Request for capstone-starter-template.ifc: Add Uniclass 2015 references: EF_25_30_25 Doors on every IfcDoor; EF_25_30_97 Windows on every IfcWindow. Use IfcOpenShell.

First a look at what the model holds.

```python
import ifcopenshell

model = ifcopenshell.open("capstone-starter-template.ifc")
print(model.schema)
print("classifications:", [c.Name for c in model.by_type("IfcClassification")])
for ifc_class in ("IfcDoor", "IfcRoof", "IfcStair", "IfcWall", "IfcWindow"):
    print(ifc_class, len(model.by_type(ifc_class)))
```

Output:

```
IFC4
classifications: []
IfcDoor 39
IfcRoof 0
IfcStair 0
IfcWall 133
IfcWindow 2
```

```python
import ifcopenshell
import ifcopenshell.api.classification

model = ifcopenshell.open("capstone-starter-template.ifc")

system = ifcopenshell.api.classification.add_classification(model, classification="Uniclass 2015")

codes = {
    "IfcDoor": ("EF_25_30_25", "Doors"),
    "IfcWindow": ("EF_25_30_97", "Windows"),
}
for ifc_class, (code, name) in codes.items():
    products = model.by_type(ifc_class)
    ifcopenshell.api.classification.add_reference(
        model, products=products, classification=system, identification=code, name=name
    )
    print(code, len(products))

model.write("capstone-starter-template-out.ifc")
```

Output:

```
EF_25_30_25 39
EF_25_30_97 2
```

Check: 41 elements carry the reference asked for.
